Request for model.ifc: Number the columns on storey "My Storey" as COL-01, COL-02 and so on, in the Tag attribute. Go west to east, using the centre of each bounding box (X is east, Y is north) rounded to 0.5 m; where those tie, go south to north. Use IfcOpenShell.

First a look at what the model holds.

```python
import ifcopenshell
import ifcopenshell.util.element
import ifcopenshell.util.placement

model = ifcopenshell.open("model.ifc")
print(model.schema)
storey = next(s for s in model.by_type("IfcBuildingStorey") if s.Name == "My Storey")
columns = [e for e in ifcopenshell.util.element.get_decomposition(storey) if e.is_a("IfcColumn")]
for e in sorted(columns, key=lambda e: e.id()):
    origin = ifcopenshell.util.placement.get_local_placement(e.ObjectPlacement)[:3, 3]
    print(e.id(), e.Tag, e.Name, origin.round(2) + 0.0, sep=" | ")
```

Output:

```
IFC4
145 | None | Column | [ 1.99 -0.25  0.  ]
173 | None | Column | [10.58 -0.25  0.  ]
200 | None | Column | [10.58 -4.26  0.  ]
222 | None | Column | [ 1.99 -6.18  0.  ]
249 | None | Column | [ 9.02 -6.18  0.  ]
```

```python
import ifcopenshell
import ifcopenshell.geom
import ifcopenshell.util.element
import ifcopenshell.util.shape

model = ifcopenshell.open("model.ifc")
settings = ifcopenshell.geom.settings()
settings.set("use-world-coords", True)


def centre(element):
    shape = ifcopenshell.geom.create_shape(settings, element)
    return ifcopenshell.util.shape.get_bbox_centroid(shape.geometry)


storey = next(s for s in model.by_type("IfcBuildingStorey") if s.Name == "My Storey")
columns = [e for e in ifcopenshell.util.element.get_decomposition(storey) if e.is_a("IfcColumn")]

# Insertion points can sit at a corner or the storey origin, so sort by the geometry (in metres).
centres = {e: centre(e) for e in columns}
columns.sort(key=lambda e: (round(centres[e][0] / 0.5), centres[e][1]))

for i, e in enumerate(columns, start=1):
    number = f"COL-{i:02d}"
    e.Tag = number
    print(e.id(), number)

model.write("model-out.ifc")
```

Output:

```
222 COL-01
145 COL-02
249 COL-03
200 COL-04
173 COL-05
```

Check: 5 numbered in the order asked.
